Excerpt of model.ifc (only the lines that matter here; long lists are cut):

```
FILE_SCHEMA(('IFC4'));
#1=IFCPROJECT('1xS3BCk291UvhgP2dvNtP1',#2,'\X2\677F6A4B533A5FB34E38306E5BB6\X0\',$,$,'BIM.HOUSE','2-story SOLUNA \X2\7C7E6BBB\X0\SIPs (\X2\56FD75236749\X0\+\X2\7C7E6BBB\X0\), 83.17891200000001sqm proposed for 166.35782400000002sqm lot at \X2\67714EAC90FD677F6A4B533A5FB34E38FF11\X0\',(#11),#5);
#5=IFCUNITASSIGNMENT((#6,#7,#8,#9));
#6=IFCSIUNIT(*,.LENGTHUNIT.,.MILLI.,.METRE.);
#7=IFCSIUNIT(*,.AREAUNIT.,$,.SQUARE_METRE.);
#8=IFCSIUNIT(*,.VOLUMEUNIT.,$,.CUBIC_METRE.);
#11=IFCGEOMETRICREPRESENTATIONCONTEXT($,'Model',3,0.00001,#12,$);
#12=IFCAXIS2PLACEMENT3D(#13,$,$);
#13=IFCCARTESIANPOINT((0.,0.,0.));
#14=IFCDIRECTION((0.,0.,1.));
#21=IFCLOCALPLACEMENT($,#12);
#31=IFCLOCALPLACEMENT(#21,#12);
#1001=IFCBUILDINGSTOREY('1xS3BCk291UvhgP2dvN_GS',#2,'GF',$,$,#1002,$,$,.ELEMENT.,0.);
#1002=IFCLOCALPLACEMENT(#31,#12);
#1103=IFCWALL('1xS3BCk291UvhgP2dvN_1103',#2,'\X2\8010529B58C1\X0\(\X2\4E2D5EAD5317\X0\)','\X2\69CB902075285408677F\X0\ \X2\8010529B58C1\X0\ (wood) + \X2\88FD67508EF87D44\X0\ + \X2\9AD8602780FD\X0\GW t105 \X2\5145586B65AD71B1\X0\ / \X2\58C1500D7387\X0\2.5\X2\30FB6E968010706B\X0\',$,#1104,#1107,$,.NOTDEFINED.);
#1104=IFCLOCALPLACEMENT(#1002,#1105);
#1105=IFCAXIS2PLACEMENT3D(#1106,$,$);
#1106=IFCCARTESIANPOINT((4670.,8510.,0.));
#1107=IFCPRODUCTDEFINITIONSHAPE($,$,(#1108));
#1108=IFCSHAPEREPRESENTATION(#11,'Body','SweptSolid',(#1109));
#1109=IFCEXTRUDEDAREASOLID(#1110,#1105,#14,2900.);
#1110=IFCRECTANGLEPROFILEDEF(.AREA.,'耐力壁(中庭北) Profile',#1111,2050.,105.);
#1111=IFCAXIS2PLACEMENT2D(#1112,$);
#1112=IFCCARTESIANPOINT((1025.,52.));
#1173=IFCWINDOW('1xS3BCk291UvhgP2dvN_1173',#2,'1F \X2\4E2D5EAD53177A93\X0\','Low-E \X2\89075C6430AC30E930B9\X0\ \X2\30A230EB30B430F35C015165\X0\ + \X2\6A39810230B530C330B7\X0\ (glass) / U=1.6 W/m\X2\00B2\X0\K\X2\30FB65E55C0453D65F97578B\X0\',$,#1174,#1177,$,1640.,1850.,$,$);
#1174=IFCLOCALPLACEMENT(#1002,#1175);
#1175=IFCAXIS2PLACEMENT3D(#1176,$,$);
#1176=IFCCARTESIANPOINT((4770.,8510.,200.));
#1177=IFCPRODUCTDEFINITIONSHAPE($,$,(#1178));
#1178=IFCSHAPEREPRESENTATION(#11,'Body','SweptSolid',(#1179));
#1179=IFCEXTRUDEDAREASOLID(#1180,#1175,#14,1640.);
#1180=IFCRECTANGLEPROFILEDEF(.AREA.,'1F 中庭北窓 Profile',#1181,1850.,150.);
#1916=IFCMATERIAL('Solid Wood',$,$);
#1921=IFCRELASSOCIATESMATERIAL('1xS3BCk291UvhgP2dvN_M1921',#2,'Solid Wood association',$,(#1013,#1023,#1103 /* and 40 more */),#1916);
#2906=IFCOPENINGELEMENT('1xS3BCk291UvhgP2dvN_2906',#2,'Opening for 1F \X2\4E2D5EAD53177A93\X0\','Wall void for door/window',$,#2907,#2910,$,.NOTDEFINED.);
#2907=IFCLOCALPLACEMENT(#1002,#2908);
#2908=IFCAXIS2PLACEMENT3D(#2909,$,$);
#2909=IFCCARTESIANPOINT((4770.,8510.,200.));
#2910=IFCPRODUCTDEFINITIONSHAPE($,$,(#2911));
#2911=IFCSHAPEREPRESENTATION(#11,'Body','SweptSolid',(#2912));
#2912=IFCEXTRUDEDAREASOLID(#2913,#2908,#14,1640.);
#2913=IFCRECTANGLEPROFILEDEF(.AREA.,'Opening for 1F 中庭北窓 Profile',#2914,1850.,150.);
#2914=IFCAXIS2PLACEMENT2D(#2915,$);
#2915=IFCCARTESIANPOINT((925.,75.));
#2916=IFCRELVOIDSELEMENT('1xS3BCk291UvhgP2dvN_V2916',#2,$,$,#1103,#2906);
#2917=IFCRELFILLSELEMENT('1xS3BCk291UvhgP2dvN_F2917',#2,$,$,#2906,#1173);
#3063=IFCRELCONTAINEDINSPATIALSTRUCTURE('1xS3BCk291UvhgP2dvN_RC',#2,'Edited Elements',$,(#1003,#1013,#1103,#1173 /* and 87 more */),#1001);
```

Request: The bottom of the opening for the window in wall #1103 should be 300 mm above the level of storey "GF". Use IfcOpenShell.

```python
import numpy as np
import ifcopenshell
import ifcopenshell.api.geometry
import ifcopenshell.geom
import ifcopenshell.util.element
import ifcopenshell.util.placement
import ifcopenshell.util.shape
import ifcopenshell.util.unit

model = ifcopenshell.open("model.ifc")
unit_scale = ifcopenshell.util.unit.calculate_unit_scale(model)

window = model.by_id(1173)
opening = window.FillsVoids[0].RelatingOpeningElement
storey = ifcopenshell.util.element.get_container(window, ifc_class="IfcBuildingStorey")
level = ifcopenshell.util.placement.get_local_placement(storey.ObjectPlacement)[2, 3]

# The opening's origin need not be at the sill, so measure its lowest point.
shape = ifcopenshell.geom.create_shape(ifcopenshell.geom.settings(), opening)
bottom = ifcopenshell.util.shape.get_shape_bottom_elevation(shape, shape.geometry) / unit_scale
dz = level + 0.3 / unit_scale - bottom

shift = np.array([0.0, 0.0, dz])
# The window is not placed relative to its opening, so move both.
for product in (opening, window):
    matrix = ifcopenshell.util.placement.get_local_placement(product.ObjectPlacement)
    matrix[:3, 3] += shift
    ifcopenshell.api.geometry.edit_object_placement(model, product=product, matrix=matrix, is_si=False)

print(f"moved by {dz * unit_scale:+.3f} m")

model.write("model_updated.ifc")
```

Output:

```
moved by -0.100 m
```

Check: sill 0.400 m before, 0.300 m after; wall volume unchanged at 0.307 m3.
